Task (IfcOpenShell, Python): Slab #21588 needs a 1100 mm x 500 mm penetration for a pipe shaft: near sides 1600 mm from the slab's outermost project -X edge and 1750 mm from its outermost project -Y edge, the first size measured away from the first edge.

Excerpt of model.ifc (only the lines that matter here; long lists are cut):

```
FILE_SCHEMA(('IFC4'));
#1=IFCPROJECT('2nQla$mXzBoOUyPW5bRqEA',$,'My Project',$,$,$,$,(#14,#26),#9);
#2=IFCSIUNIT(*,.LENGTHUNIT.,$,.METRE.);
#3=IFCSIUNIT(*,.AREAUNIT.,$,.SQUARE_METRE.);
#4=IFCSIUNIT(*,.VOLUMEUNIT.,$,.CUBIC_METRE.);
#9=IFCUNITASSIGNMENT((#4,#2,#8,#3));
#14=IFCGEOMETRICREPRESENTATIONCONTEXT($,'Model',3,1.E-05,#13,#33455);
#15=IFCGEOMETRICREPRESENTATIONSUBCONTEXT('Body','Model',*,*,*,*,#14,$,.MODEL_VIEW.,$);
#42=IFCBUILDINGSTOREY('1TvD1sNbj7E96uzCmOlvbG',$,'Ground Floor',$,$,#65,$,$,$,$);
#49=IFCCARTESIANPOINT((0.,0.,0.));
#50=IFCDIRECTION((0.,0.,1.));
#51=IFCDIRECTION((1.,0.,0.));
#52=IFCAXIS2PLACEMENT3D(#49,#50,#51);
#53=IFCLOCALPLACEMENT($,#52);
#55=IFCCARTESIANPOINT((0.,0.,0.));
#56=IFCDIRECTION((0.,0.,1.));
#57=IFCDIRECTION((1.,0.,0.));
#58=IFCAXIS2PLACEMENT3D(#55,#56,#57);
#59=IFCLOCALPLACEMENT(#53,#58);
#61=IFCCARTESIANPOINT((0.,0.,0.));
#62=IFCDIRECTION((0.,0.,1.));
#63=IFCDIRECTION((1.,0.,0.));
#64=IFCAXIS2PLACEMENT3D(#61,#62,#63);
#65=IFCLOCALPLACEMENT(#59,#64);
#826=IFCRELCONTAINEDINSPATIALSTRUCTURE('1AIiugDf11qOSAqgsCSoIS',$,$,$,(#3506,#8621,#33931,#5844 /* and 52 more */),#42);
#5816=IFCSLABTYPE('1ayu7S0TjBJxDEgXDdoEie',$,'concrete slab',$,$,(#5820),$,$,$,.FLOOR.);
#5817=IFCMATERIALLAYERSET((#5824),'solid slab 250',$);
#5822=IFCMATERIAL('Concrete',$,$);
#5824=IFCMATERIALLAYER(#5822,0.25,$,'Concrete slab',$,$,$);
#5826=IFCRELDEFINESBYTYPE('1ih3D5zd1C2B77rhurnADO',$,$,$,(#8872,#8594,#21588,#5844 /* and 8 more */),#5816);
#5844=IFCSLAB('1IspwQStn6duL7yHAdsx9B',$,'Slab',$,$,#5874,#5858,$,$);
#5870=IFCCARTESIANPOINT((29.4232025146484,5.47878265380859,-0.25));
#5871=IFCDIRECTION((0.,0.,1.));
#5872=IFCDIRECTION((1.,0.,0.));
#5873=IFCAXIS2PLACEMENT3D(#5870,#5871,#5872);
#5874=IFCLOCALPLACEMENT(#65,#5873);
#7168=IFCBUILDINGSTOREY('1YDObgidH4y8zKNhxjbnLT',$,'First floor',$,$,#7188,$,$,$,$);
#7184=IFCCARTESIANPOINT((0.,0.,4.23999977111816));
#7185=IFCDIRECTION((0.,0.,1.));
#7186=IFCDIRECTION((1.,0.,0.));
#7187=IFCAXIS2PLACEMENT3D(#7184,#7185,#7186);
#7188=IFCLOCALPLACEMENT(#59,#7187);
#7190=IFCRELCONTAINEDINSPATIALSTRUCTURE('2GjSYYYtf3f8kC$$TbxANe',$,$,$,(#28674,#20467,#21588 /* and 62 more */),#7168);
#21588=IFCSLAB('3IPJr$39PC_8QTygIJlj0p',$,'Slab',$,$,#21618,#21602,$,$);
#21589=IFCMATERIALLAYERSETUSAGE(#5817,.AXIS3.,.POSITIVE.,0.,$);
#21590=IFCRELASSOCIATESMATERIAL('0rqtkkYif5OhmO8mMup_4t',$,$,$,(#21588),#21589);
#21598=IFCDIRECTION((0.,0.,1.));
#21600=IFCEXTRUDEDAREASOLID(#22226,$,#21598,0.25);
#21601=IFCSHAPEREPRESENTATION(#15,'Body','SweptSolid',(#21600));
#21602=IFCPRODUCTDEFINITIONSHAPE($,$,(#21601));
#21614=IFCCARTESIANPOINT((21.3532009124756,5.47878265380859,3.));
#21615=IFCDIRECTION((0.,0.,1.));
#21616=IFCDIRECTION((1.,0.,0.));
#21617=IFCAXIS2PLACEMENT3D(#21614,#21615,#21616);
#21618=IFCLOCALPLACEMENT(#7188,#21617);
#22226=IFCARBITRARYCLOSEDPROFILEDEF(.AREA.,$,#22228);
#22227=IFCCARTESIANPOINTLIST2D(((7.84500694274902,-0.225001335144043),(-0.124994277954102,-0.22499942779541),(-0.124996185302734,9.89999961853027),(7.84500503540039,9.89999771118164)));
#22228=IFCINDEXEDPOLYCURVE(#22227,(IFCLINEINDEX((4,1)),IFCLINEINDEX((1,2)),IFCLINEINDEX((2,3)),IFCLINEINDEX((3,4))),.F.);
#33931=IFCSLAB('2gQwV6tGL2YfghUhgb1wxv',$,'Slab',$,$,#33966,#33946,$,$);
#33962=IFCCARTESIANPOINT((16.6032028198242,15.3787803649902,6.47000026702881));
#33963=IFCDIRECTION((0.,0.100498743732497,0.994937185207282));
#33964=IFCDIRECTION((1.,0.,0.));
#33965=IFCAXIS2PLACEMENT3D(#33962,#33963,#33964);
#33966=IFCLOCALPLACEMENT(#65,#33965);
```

```python
import numpy as np
import ifcopenshell
import ifcopenshell.api.feature
import ifcopenshell.api.geometry
import ifcopenshell.api.root
import ifcopenshell.geom
import ifcopenshell.util.placement
import ifcopenshell.util.representation
import ifcopenshell.util.shape
import ifcopenshell.util.unit

model = ifcopenshell.open("model.ifc")
unit_scale = ifcopenshell.util.unit.calculate_unit_scale(model)
settings = ifcopenshell.geom.settings()


def volume(element):
    """Net volume in cubic metres, openings subtracted."""
    shape = ifcopenshell.geom.create_shape(settings, element)
    return ifcopenshell.util.shape.get_volume(shape.geometry)


slab = model.by_guid("3IPJr$39PC_8QTygIJlj0p")
before = volume(slab)

# Extent in the slab's own axes, in metres. The edges named are its -X and -Y sides.
slab_shape = ifcopenshell.geom.create_shape(settings, slab)
vertices = ifcopenshell.util.shape.get_vertices(slab_shape.geometry)
x_min, y_min, bottom = vertices.min(axis=0)
top = vertices[:, 2].max()

opening = ifcopenshell.api.root.create_entity(model, ifc_class="IfcOpeningElement", name="Pipe shaft opening", predefined_type="OPENING")
context = ifcopenshell.util.representation.get_context(model, "Model", "Body", "MODEL_VIEW")
width, depth = 1.1, 0.5
outline = [(0.0, 0.0), (width, 0.0), (width, depth), (0.0, depth), (0.0, 0.0)]
# Overshoot both faces by 50 mm so the cut is clean.
shape = ifcopenshell.api.geometry.add_slab_representation(
    model, context=context, depth=top - bottom + 0.1, polyline=outline
)
ifcopenshell.api.geometry.assign_representation(model, product=opening, representation=shape)

matrix = ifcopenshell.util.placement.get_local_placement(slab.ObjectPlacement)
matrix[:, 3] = matrix @ np.append(np.array([x_min + 1.6, y_min + 1.75, bottom - 0.05]) / unit_scale, 1.0)
ifcopenshell.api.geometry.edit_object_placement(model, product=opening, matrix=matrix, is_si=False)
ifcopenshell.api.feature.add_feature(model, feature=opening, element=slab)

after = volume(slab)

print(f"slab volume {before:.3f} -> {after:.3f} m3")

model.write("model_edited.ifc")
```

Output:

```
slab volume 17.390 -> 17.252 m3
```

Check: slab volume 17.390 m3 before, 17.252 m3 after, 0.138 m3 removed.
